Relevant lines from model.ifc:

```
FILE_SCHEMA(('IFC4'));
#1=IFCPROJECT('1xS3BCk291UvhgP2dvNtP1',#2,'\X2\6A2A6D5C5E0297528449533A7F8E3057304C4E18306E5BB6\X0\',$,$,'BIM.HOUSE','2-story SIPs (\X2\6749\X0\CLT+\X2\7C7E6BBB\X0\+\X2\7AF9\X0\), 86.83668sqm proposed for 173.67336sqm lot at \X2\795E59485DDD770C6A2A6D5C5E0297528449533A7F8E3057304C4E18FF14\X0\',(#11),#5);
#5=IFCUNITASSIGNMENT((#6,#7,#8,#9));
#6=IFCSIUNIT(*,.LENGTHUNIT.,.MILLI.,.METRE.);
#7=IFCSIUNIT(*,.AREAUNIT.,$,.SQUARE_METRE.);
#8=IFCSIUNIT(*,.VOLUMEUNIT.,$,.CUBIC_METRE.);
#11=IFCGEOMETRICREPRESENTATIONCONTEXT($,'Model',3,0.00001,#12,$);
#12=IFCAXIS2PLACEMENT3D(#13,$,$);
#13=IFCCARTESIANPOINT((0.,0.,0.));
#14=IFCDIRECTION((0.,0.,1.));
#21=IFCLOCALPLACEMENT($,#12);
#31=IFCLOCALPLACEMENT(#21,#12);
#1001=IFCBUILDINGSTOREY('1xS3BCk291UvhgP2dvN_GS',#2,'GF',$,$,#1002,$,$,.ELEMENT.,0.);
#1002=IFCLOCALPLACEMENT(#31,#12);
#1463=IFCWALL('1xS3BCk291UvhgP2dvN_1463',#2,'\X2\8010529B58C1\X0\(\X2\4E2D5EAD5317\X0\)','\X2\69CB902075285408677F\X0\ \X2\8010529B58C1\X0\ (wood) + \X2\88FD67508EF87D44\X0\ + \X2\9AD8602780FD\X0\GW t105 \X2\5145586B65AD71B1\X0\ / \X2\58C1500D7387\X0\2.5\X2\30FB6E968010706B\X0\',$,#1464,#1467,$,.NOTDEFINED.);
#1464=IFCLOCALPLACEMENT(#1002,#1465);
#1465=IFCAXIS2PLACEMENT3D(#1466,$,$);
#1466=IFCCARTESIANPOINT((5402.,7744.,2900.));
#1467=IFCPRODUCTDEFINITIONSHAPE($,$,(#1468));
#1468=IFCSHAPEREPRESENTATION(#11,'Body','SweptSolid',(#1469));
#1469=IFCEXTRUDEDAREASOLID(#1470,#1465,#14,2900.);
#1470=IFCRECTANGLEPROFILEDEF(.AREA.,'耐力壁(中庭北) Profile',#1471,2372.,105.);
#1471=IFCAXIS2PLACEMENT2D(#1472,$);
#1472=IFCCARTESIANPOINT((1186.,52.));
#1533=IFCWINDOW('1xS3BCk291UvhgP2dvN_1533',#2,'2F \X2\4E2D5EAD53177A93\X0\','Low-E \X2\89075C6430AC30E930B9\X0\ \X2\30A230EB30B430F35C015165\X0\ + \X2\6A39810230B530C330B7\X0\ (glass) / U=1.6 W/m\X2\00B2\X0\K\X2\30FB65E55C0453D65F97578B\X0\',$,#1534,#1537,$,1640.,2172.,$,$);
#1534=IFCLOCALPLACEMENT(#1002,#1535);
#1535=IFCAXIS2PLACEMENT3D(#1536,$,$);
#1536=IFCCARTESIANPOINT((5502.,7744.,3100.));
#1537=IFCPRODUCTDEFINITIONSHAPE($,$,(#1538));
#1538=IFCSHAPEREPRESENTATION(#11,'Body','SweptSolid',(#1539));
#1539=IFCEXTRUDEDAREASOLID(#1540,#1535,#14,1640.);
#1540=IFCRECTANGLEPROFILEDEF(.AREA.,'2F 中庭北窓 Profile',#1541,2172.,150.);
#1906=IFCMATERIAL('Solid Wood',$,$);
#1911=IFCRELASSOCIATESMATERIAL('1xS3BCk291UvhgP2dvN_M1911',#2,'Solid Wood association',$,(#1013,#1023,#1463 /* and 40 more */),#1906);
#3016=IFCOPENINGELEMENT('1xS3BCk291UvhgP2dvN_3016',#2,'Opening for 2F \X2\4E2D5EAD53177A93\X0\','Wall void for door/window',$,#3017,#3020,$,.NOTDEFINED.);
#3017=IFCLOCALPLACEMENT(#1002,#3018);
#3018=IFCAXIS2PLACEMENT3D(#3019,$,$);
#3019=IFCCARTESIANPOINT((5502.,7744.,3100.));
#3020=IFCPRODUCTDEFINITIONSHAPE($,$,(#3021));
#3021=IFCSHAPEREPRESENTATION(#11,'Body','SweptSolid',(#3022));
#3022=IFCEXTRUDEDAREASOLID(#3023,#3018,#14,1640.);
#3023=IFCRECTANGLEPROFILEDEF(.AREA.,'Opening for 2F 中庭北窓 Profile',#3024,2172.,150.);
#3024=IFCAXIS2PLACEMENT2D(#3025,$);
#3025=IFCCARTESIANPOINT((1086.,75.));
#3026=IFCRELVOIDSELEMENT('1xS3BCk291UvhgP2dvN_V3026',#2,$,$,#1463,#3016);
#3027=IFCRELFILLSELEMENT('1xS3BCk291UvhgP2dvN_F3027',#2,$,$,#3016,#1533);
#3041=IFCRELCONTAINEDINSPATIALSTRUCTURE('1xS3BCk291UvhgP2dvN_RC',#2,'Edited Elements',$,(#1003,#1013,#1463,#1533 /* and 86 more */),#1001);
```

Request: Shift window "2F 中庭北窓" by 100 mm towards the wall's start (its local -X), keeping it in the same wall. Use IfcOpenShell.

```python
import ifcopenshell
import ifcopenshell.api.geometry
import ifcopenshell.util.placement
import ifcopenshell.util.unit

model = ifcopenshell.open("model.ifc")
unit_scale = ifcopenshell.util.unit.calculate_unit_scale(model)

window = model.by_id(1533)
opening = window.FillsVoids[0].RelatingOpeningElement
wall = opening.VoidsElements[0].RelatingBuildingElement

wall_matrix = ifcopenshell.util.placement.get_local_placement(wall.ObjectPlacement)
shift = wall_matrix[:3, 0] * -0.1 / unit_scale
before = ifcopenshell.util.placement.get_local_placement(window.ObjectPlacement)[:3, 3].copy()

# The window is not placed relative to its opening, so move both.
for product in (opening, window):
    matrix = ifcopenshell.util.placement.get_local_placement(product.ObjectPlacement)
    matrix[:3, 3] += shift
    ifcopenshell.api.geometry.edit_object_placement(model, product=product, matrix=matrix, is_si=False)

after = ifcopenshell.util.placement.get_local_placement(window.ObjectPlacement)[:3, 3]
print("window moved by", (after - before).round(3) + 0.0)

model.write("model_rev.ifc")
```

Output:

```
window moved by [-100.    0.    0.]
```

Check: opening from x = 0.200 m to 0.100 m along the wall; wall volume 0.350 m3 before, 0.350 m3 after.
